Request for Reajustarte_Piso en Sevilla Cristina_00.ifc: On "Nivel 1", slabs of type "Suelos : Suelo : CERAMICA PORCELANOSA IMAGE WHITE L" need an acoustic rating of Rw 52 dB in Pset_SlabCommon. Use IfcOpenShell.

First a look at what the model holds.

```python
import ifcopenshell
import ifcopenshell.util.element

model = ifcopenshell.open("Reajustarte_Piso en Sevilla Cristina_00.ifc")
print(model.schema)
storey = next(s for s in model.by_type("IfcBuildingStorey") if s.Name == "Nivel 1")
slabs = [e for e in ifcopenshell.util.element.get_decomposition(storey) if e.is_a("IfcSlab")]
seen = {}
for e in slabs:
    element_type = ifcopenshell.util.element.get_type(e)
    key = (element_type.Name if element_type != e and element_type else None, ifcopenshell.util.element.get_pset(e, "Pset_SlabCommon", "AcousticRating"))
    seen[key] = seen.get(key, 0) + 1
for (name, value), count in sorted(seen.items(), key=str):
    print(count, "x", name, "|", value)
```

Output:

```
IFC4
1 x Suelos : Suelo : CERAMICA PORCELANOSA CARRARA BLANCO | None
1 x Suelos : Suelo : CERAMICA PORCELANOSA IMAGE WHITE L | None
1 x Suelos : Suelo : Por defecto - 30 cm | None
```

```python
import ifcopenshell
import ifcopenshell.api.pset
import ifcopenshell.util.element

model = ifcopenshell.open("Reajustarte_Piso en Sevilla Cristina_00.ifc")

storey = next(s for s in model.by_type("IfcBuildingStorey") if s.Name == "Nivel 1")
slabs = [e for e in ifcopenshell.util.element.get_decomposition(storey) if e.is_a("IfcSlab")]

count = 0
for e in slabs:
    element_type = ifcopenshell.util.element.get_type(e)
    if element_type in (None, e) or element_type.Name != "Suelos : Suelo : CERAMICA PORCELANOSA IMAGE WHITE L":
        continue
    # add_pset returns the element's existing set when there is one.
    pset = ifcopenshell.api.pset.add_pset(model, product=e, name="Pset_SlabCommon")
    ifcopenshell.api.pset.edit_pset(model, pset=pset, properties={"AcousticRating": "Rw 52 dB"})
    count += 1

print(count, "slabs updated")

model.write("Reajustarte_Piso en Sevilla Cristina_00_edited.ifc")
```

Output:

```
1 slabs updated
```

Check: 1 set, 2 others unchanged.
